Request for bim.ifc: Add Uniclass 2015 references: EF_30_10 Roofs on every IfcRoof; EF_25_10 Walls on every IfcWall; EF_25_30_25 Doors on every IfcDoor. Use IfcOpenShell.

First a look at what the model holds.

```python
import ifcopenshell

model = ifcopenshell.open("bim.ifc")
print(model.schema)
print("classifications:", [c.Name for c in model.by_type("IfcClassification")])
for ifc_class in ("IfcDoor", "IfcRoof", "IfcStair", "IfcWall", "IfcWindow"):
    print(ifc_class, len(model.by_type(ifc_class)))
```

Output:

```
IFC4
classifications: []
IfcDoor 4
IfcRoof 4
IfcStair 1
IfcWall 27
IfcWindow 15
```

```python
import ifcopenshell
import ifcopenshell.api.classification

model = ifcopenshell.open("bim.ifc")

system = ifcopenshell.api.classification.add_classification(model, classification="Uniclass 2015")

codes = {
    "IfcRoof": ("EF_30_10", "Roofs"),
    "IfcWall": ("EF_25_10", "Walls"),
    "IfcDoor": ("EF_25_30_25", "Doors"),
}
for ifc_class, (code, name) in codes.items():
    products = model.by_type(ifc_class)
    ifcopenshell.api.classification.add_reference(
        model, products=products, classification=system, identification=code, name=name
    )
    print(code, len(products))

model.write("bim_v2.ifc")
```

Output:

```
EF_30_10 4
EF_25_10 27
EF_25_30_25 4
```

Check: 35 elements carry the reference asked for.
